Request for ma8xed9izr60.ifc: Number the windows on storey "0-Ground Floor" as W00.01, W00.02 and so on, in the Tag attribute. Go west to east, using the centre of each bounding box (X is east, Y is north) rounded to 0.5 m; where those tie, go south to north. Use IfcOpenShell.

First a look at what the model holds.

```python
import ifcopenshell
import ifcopenshell.util.element
import ifcopenshell.util.placement

model = ifcopenshell.open("ma8xed9izr60.ifc")
print(model.schema)
storey = next(s for s in model.by_type("IfcBuildingStorey") if s.Name == "0-Ground Floor")
windows = [e for e in ifcopenshell.util.element.get_decomposition(storey) if e.is_a("IfcWindow")]
for e in sorted(windows, key=lambda e: e.id()):
    origin = ifcopenshell.util.placement.get_local_placement(e.ObjectPlacement)[:3, 3]
    print(e.id(), e.Tag, e.Name, origin.round(2) + 0.0, sep=" | ")
```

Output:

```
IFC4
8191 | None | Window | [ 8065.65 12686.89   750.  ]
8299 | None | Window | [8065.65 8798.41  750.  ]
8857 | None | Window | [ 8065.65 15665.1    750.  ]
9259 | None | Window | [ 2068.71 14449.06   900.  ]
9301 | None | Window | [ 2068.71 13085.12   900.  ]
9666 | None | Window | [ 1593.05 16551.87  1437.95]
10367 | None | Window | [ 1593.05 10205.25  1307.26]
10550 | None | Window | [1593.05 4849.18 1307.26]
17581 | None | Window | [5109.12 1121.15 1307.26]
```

```python
import ifcopenshell
import ifcopenshell.geom
import ifcopenshell.util.element
import ifcopenshell.util.shape

model = ifcopenshell.open("ma8xed9izr60.ifc")
settings = ifcopenshell.geom.settings()
settings.set("use-world-coords", True)


def centre(element):
    shape = ifcopenshell.geom.create_shape(settings, element)
    return ifcopenshell.util.shape.get_bbox_centroid(shape.geometry)


storey = next(s for s in model.by_type("IfcBuildingStorey") if s.Name == "0-Ground Floor")
windows = [e for e in ifcopenshell.util.element.get_decomposition(storey) if e.is_a("IfcWindow")]

# Insertion points can sit at a corner or the storey origin, so sort by the geometry (in metres).
centres = {e: centre(e) for e in windows}
windows.sort(key=lambda e: (round(centres[e][0] / 0.5), centres[e][1]))

for i, e in enumerate(windows, start=1):
    number = f"W00.{i:02d}"
    e.Tag = number
    print(e.id(), number)

model.write("ma8xed9izr60_edited.ifc")
```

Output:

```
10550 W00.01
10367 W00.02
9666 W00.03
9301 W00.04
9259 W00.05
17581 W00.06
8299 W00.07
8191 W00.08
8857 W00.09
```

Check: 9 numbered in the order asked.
